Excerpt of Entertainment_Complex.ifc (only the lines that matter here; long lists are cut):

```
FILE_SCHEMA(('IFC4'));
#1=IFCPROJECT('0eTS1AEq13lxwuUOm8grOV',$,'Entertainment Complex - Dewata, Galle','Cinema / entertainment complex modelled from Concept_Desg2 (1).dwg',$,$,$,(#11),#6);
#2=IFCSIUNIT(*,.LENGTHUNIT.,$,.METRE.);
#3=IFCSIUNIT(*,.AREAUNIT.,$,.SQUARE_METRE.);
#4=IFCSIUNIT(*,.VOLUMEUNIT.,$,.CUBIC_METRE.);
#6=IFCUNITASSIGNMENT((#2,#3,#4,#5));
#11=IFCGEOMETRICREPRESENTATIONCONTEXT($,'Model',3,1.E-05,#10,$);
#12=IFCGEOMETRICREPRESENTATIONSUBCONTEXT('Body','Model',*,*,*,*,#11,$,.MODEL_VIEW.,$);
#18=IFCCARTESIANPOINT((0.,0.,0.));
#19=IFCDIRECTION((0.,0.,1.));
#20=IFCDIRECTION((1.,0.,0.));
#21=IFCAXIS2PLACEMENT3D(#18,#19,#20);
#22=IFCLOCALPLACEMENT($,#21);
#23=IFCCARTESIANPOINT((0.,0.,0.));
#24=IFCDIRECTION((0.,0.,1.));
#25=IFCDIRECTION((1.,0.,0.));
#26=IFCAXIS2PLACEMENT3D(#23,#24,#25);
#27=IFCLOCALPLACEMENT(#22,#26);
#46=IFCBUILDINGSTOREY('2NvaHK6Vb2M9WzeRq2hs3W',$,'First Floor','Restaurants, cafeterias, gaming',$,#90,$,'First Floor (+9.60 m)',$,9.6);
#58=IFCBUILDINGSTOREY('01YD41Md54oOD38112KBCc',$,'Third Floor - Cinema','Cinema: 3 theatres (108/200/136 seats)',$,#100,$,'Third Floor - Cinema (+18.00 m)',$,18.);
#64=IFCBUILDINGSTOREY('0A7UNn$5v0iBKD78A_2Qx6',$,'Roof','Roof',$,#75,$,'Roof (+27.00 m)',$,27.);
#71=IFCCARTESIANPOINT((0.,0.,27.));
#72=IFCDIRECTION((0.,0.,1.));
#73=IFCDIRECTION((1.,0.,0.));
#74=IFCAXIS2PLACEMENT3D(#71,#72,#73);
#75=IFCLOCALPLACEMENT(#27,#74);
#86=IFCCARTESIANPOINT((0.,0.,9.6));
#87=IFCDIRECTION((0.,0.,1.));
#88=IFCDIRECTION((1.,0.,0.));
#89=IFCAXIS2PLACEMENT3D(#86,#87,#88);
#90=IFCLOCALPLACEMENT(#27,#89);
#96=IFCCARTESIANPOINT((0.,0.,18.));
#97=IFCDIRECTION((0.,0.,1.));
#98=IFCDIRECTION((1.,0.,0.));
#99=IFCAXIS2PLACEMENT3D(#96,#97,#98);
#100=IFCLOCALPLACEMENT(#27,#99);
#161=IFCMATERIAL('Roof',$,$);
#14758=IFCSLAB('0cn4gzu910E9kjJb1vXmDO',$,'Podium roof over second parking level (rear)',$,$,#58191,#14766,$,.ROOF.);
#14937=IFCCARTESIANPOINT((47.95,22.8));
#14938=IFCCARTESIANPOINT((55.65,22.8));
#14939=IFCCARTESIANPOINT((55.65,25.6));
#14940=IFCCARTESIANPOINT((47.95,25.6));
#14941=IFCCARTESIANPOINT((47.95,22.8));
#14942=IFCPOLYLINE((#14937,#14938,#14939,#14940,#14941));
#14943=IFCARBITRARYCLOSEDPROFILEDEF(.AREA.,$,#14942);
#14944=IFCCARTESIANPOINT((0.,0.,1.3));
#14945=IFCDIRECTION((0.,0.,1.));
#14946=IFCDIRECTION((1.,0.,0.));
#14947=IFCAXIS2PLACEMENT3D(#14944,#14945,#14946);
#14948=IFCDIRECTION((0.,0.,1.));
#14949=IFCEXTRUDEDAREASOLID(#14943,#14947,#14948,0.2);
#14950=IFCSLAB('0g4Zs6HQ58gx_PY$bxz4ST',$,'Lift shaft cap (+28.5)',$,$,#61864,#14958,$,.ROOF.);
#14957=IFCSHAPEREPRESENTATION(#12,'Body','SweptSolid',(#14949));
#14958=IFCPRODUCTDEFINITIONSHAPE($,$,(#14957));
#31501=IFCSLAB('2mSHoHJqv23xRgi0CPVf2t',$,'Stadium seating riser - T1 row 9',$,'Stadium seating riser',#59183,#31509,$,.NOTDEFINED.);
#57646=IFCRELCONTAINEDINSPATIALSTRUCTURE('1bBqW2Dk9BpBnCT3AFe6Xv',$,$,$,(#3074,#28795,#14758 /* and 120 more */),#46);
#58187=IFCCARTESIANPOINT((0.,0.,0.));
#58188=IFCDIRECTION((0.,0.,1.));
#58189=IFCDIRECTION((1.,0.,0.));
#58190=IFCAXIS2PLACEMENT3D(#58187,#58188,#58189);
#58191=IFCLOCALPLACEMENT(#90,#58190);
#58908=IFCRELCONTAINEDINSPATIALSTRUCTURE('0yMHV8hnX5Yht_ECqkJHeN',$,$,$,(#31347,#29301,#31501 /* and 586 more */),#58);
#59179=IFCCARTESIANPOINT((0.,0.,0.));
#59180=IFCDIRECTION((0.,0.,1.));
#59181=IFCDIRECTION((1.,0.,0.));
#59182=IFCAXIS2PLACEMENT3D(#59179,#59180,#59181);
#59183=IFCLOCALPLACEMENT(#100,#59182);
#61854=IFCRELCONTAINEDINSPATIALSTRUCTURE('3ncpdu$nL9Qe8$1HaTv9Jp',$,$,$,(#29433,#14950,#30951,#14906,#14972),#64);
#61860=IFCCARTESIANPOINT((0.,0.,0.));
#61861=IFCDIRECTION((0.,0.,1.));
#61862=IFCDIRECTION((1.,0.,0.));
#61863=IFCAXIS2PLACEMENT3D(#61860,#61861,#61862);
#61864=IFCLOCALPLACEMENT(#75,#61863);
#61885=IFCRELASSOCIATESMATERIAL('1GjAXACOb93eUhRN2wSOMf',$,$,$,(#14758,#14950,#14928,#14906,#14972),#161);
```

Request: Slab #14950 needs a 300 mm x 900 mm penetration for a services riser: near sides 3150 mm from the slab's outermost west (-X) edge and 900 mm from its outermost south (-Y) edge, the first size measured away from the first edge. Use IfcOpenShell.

```python
import numpy as np
import ifcopenshell
import ifcopenshell.api.feature
import ifcopenshell.api.geometry
import ifcopenshell.api.root
import ifcopenshell.geom
import ifcopenshell.util.placement
import ifcopenshell.util.representation
import ifcopenshell.util.shape
import ifcopenshell.util.unit

model = ifcopenshell.open("Entertainment_Complex.ifc")
unit_scale = ifcopenshell.util.unit.calculate_unit_scale(model)
settings = ifcopenshell.geom.settings()


def volume(element):
    """Net volume in cubic metres, openings subtracted."""
    shape = ifcopenshell.geom.create_shape(settings, element)
    return ifcopenshell.util.shape.get_volume(shape.geometry)


slab = model.by_guid("0g4Zs6HQ58gx_PY$bxz4ST")
before = volume(slab)

# Extent in the slab's own axes, in metres. The edges named are its -X and -Y sides.
slab_shape = ifcopenshell.geom.create_shape(settings, slab)
vertices = ifcopenshell.util.shape.get_vertices(slab_shape.geometry)
x_min, y_min, bottom = vertices.min(axis=0)
top = vertices[:, 2].max()

opening = ifcopenshell.api.root.create_entity(model, ifc_class="IfcOpeningElement", name="Services riser opening", predefined_type="OPENING")
context = ifcopenshell.util.representation.get_context(model, "Model", "Body", "MODEL_VIEW")
width, depth = 0.3, 0.9
outline = [(0.0, 0.0), (width, 0.0), (width, depth), (0.0, depth), (0.0, 0.0)]
# Overshoot both faces by 50 mm so the cut is clean.
shape = ifcopenshell.api.geometry.add_slab_representation(
    model, context=context, depth=top - bottom + 0.1, polyline=outline
)
ifcopenshell.api.geometry.assign_representation(model, product=opening, representation=shape)

matrix = ifcopenshell.util.placement.get_local_placement(slab.ObjectPlacement)
matrix[:, 3] = matrix @ np.append(np.array([x_min + 3.15, y_min + 0.9, bottom - 0.05]) / unit_scale, 1.0)
ifcopenshell.api.geometry.edit_object_placement(model, product=opening, matrix=matrix, is_si=False)
ifcopenshell.api.feature.add_feature(model, feature=opening, element=slab)

after = volume(slab)

print(f"slab volume {before:.3f} -> {after:.3f} m3")

model.write("Entertainment_Complex_rev.ifc")
```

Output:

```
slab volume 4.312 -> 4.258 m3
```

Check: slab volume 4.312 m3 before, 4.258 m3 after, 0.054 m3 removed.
